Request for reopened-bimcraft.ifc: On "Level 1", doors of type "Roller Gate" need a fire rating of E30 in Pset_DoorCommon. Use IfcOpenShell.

First a look at what the model holds.

```python
import ifcopenshell
import ifcopenshell.util.element

model = ifcopenshell.open("reopened-bimcraft.ifc")
print(model.schema)
storey = next(s for s in model.by_type("IfcBuildingStorey") if s.Name == "Level 1")
doors = [e for e in ifcopenshell.util.element.get_decomposition(storey) if e.is_a("IfcDoor")]
seen = {}
for e in doors:
    element_type = ifcopenshell.util.element.get_type(e)
    key = (element_type.Name if element_type != e and element_type else None, ifcopenshell.util.element.get_pset(e, "Pset_DoorCommon", "FireRating"))
    seen[key] = seen.get(key, 0) + 1
for (name, value), count in sorted(seen.items(), key=str):
    print(count, "x", name, "|", value)
```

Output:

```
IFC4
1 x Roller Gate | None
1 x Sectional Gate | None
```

```python
import ifcopenshell
import ifcopenshell.api.pset
import ifcopenshell.util.element

model = ifcopenshell.open("reopened-bimcraft.ifc")

storey = next(s for s in model.by_type("IfcBuildingStorey") if s.Name == "Level 1")
doors = [e for e in ifcopenshell.util.element.get_decomposition(storey) if e.is_a("IfcDoor")]

count = 0
for e in doors:
    element_type = ifcopenshell.util.element.get_type(e)
    if element_type in (None, e) or element_type.Name != "Roller Gate":
        continue
    # add_pset returns the element's existing set when there is one.
    pset = ifcopenshell.api.pset.add_pset(model, product=e, name="Pset_DoorCommon")
    ifcopenshell.api.pset.edit_pset(model, pset=pset, properties={"FireRating": "E30"})
    count += 1

print(count, "doors updated")

model.write("reopened-bimcraft_v2.ifc")
```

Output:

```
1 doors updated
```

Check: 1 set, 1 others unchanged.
